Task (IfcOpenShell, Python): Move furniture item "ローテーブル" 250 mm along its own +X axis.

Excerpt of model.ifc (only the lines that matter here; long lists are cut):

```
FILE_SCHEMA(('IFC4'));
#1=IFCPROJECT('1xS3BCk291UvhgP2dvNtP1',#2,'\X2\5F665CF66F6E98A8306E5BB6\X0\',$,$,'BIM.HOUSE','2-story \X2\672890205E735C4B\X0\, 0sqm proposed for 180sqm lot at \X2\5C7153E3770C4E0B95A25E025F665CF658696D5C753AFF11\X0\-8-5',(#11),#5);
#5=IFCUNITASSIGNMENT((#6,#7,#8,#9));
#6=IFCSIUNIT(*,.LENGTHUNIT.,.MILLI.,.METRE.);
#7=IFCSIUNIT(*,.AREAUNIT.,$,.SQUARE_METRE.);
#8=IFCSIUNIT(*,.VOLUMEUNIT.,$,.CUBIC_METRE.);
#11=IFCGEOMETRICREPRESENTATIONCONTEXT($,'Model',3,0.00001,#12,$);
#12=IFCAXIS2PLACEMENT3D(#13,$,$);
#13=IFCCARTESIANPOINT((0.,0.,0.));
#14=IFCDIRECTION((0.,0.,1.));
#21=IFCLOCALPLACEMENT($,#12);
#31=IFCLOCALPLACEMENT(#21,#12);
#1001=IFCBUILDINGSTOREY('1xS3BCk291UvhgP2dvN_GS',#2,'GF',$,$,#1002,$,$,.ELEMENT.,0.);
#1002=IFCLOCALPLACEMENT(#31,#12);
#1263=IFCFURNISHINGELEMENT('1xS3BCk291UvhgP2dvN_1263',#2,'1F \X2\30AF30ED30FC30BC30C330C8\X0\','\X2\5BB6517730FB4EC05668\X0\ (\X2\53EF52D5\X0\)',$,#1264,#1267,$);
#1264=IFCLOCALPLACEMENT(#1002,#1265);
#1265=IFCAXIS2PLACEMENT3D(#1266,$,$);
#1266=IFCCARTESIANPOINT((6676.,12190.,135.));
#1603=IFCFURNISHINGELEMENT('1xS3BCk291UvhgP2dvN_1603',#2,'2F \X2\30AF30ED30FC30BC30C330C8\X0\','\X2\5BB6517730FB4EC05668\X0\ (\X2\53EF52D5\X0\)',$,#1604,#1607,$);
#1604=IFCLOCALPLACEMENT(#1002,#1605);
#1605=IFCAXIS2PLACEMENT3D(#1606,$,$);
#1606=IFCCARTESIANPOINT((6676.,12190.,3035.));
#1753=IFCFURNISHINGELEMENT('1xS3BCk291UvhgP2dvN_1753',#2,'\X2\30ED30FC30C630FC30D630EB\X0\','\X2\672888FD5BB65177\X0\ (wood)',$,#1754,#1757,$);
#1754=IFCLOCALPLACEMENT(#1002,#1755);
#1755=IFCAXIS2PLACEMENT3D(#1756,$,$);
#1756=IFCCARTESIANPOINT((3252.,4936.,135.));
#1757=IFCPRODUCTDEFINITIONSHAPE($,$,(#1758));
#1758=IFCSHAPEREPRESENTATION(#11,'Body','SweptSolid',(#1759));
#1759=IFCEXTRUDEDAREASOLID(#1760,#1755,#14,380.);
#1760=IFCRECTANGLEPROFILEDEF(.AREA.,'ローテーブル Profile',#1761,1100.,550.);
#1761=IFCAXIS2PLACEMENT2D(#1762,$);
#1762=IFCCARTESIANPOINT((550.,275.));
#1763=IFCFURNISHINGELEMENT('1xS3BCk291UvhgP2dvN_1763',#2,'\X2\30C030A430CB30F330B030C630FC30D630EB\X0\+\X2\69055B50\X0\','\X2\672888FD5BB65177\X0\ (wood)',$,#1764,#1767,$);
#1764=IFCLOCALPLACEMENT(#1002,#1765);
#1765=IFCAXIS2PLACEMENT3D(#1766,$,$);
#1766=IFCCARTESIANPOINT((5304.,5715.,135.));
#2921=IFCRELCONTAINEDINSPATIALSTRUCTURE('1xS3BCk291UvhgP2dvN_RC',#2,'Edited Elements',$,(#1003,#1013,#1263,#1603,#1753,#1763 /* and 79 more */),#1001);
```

```python
import ifcopenshell
import ifcopenshell.api.geometry
import ifcopenshell.util.placement
import ifcopenshell.util.unit

model = ifcopenshell.open("model.ifc")
unit_scale = ifcopenshell.util.unit.calculate_unit_scale(model)

item = model.by_guid("1xS3BCk291UvhgP2dvN_1753")
matrix = ifcopenshell.util.placement.get_local_placement(item.ObjectPlacement)
matrix[:3, 3] += matrix[:3, 0] * 0.25 / unit_scale
ifcopenshell.api.geometry.edit_object_placement(model, product=item, matrix=matrix, is_si=False)

print(ifcopenshell.util.placement.get_local_placement(item.ObjectPlacement).round(3) + 0.0)

model.write("model_rev.ifc")
```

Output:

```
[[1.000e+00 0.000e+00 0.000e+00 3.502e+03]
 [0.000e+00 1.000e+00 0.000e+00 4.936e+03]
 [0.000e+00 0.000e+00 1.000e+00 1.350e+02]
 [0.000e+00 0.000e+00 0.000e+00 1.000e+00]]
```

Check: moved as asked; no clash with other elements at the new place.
